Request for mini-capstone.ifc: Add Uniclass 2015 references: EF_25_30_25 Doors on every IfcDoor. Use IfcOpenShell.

First a look at what the model holds.

```python
import ifcopenshell

model = ifcopenshell.open("mini-capstone.ifc")
print(model.schema)
print("classifications:", [c.Name for c in model.by_type("IfcClassification")])
for ifc_class in ("IfcDoor", "IfcRoof", "IfcStair", "IfcWall", "IfcWindow"):
    print(ifc_class, len(model.by_type(ifc_class)))
```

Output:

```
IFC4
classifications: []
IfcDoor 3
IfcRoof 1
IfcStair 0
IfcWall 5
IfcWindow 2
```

```python
import ifcopenshell
import ifcopenshell.api.classification

model = ifcopenshell.open("mini-capstone.ifc")

system = ifcopenshell.api.classification.add_classification(model, classification="Uniclass 2015")

codes = {
    "IfcDoor": ("EF_25_30_25", "Doors"),
}
for ifc_class, (code, name) in codes.items():
    products = model.by_type(ifc_class)
    ifcopenshell.api.classification.add_reference(
        model, products=products, classification=system, identification=code, name=name
    )
    print(code, len(products))

model.write("mini-capstone-out.ifc")
```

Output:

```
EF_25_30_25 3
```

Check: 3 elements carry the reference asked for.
